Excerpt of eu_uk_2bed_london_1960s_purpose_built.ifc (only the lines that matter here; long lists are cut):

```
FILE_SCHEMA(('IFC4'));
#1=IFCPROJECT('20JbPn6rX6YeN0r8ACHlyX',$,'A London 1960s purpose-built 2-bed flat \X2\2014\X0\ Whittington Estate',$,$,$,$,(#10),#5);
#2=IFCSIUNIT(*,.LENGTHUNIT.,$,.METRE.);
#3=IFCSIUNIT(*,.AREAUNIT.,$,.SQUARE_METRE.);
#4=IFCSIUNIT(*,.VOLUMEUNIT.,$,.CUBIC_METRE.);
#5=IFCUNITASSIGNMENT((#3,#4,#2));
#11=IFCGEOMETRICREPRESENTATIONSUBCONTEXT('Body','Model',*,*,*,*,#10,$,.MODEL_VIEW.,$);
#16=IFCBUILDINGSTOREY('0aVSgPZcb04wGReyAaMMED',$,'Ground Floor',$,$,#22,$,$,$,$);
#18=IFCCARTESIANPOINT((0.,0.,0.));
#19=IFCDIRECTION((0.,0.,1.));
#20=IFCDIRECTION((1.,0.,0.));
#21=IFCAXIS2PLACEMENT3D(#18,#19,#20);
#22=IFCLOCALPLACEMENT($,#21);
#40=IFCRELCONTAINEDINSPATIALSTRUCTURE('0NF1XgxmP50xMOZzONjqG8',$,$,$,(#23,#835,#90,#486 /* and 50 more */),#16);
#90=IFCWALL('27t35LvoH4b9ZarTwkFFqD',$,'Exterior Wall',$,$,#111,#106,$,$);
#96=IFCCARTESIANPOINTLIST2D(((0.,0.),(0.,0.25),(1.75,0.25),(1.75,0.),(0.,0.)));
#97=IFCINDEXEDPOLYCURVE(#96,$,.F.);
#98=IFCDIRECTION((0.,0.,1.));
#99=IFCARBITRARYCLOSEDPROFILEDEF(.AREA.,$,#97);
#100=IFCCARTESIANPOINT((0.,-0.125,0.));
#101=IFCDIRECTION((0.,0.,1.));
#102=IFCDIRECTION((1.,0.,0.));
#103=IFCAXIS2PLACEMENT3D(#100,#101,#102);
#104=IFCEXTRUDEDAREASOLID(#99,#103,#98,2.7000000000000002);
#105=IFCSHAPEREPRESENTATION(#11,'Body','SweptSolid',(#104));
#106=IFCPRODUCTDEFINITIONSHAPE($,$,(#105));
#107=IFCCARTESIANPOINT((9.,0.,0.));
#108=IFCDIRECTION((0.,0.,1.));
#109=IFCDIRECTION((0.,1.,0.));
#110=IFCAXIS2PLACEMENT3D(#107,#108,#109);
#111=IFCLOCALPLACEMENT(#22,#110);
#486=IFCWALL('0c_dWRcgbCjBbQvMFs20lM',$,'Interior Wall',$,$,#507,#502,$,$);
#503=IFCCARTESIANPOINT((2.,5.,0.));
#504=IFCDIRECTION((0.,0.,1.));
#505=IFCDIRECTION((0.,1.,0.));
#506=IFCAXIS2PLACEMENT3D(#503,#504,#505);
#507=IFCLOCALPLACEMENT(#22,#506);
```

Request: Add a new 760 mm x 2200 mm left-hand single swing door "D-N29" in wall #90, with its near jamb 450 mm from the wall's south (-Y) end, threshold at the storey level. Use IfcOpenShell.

```python
import numpy as np
import ifcopenshell
import ifcopenshell.api.feature
import ifcopenshell.api.geometry
import ifcopenshell.api.root
import ifcopenshell.api.spatial
import ifcopenshell.geom
import ifcopenshell.util.element
import ifcopenshell.util.placement
import ifcopenshell.util.representation
import ifcopenshell.util.shape
import ifcopenshell.util.unit

model = ifcopenshell.open("eu_uk_2bed_london_1960s_purpose_built.ifc")
unit_scale = ifcopenshell.util.unit.calculate_unit_scale(model)
settings = ifcopenshell.geom.settings()


def volume(element):
    """Net volume in cubic metres, openings subtracted."""
    shape = ifcopenshell.geom.create_shape(settings, element)
    return ifcopenshell.util.shape.get_volume(shape.geometry)


wall = model.by_id(90)
storey = ifcopenshell.util.element.get_container(wall, ifc_class="IfcBuildingStorey")
context = ifcopenshell.util.representation.get_context(model, "Model", "Body", "MODEL_VIEW")
before = volume(wall)

width, height, from_end, sill = 0.76, 2.2, 0.45, 0.0  # metres

# The wall runs along its own X axis, and the end named is its -X end.
wall_shape = ifcopenshell.geom.create_shape(settings, wall)
x, y, z = ifcopenshell.util.shape.get_vertices(wall_shape.geometry).T
start = x.min() + from_end
face, thickness = float(y.min()), float(y.max() - y.min())
wall_matrix = ifcopenshell.util.placement.get_local_placement(wall.ObjectPlacement)
level = ifcopenshell.util.placement.get_local_placement(storey.ObjectPlacement)[2, 3]


def in_wall(x, y):
    """Placement at x, y metres in the wall's axes, at sill height."""
    matrix = wall_matrix.copy()
    matrix[:, 3] = wall_matrix @ np.array([x / unit_scale, y / unit_scale, 0.0, 1.0])
    matrix[2, 3] = level + sill / unit_scale
    return matrix


# Opening: a box that overshoots both wall faces by 50 mm.
opening = ifcopenshell.api.root.create_entity(model, ifc_class="IfcOpeningElement", predefined_type="OPENING")
box = ifcopenshell.api.geometry.add_wall_representation(
    model, context=context, length=width, height=height, thickness=thickness + 0.1
)
ifcopenshell.api.geometry.assign_representation(model, product=opening, representation=box)
ifcopenshell.api.geometry.edit_object_placement(model, product=opening, matrix=in_wall(start, face - 0.05), is_si=False)
ifcopenshell.api.feature.add_feature(model, feature=opening, element=wall)

door = ifcopenshell.api.root.create_entity(model, ifc_class="IfcDoor", name="D-N29", predefined_type="DOOR")
door.OverallWidth, door.OverallHeight = width / unit_scale, height / unit_scale
door.OperationType = "SINGLE_SWING_LEFT"
body = ifcopenshell.api.geometry.add_door_representation(
    model,
    context=context,
    overall_width=door.OverallWidth,
    overall_height=door.OverallHeight,
    operation_type="SINGLE_SWING_LEFT",
    lining_properties={"LiningDepth": thickness / unit_scale, "ThresholdDepth": thickness / unit_scale},
)
ifcopenshell.api.geometry.assign_representation(model, product=door, representation=body)
ifcopenshell.api.spatial.assign_container(model, products=[door], relating_structure=storey)
ifcopenshell.api.feature.add_filling(model, opening=opening, element=door)

# The lining spans the wall, so the door starts at the wall face.
ifcopenshell.api.geometry.edit_object_placement(model, product=door, matrix=in_wall(start, face), is_si=False)

after = volume(wall)

print(f"wall volume {before:.3f} -> {after:.3f} m3")

model.write("eu_uk_2bed_london_1960s_purpose_built_rev.ifc")
```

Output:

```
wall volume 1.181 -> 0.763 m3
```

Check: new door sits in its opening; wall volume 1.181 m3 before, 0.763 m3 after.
